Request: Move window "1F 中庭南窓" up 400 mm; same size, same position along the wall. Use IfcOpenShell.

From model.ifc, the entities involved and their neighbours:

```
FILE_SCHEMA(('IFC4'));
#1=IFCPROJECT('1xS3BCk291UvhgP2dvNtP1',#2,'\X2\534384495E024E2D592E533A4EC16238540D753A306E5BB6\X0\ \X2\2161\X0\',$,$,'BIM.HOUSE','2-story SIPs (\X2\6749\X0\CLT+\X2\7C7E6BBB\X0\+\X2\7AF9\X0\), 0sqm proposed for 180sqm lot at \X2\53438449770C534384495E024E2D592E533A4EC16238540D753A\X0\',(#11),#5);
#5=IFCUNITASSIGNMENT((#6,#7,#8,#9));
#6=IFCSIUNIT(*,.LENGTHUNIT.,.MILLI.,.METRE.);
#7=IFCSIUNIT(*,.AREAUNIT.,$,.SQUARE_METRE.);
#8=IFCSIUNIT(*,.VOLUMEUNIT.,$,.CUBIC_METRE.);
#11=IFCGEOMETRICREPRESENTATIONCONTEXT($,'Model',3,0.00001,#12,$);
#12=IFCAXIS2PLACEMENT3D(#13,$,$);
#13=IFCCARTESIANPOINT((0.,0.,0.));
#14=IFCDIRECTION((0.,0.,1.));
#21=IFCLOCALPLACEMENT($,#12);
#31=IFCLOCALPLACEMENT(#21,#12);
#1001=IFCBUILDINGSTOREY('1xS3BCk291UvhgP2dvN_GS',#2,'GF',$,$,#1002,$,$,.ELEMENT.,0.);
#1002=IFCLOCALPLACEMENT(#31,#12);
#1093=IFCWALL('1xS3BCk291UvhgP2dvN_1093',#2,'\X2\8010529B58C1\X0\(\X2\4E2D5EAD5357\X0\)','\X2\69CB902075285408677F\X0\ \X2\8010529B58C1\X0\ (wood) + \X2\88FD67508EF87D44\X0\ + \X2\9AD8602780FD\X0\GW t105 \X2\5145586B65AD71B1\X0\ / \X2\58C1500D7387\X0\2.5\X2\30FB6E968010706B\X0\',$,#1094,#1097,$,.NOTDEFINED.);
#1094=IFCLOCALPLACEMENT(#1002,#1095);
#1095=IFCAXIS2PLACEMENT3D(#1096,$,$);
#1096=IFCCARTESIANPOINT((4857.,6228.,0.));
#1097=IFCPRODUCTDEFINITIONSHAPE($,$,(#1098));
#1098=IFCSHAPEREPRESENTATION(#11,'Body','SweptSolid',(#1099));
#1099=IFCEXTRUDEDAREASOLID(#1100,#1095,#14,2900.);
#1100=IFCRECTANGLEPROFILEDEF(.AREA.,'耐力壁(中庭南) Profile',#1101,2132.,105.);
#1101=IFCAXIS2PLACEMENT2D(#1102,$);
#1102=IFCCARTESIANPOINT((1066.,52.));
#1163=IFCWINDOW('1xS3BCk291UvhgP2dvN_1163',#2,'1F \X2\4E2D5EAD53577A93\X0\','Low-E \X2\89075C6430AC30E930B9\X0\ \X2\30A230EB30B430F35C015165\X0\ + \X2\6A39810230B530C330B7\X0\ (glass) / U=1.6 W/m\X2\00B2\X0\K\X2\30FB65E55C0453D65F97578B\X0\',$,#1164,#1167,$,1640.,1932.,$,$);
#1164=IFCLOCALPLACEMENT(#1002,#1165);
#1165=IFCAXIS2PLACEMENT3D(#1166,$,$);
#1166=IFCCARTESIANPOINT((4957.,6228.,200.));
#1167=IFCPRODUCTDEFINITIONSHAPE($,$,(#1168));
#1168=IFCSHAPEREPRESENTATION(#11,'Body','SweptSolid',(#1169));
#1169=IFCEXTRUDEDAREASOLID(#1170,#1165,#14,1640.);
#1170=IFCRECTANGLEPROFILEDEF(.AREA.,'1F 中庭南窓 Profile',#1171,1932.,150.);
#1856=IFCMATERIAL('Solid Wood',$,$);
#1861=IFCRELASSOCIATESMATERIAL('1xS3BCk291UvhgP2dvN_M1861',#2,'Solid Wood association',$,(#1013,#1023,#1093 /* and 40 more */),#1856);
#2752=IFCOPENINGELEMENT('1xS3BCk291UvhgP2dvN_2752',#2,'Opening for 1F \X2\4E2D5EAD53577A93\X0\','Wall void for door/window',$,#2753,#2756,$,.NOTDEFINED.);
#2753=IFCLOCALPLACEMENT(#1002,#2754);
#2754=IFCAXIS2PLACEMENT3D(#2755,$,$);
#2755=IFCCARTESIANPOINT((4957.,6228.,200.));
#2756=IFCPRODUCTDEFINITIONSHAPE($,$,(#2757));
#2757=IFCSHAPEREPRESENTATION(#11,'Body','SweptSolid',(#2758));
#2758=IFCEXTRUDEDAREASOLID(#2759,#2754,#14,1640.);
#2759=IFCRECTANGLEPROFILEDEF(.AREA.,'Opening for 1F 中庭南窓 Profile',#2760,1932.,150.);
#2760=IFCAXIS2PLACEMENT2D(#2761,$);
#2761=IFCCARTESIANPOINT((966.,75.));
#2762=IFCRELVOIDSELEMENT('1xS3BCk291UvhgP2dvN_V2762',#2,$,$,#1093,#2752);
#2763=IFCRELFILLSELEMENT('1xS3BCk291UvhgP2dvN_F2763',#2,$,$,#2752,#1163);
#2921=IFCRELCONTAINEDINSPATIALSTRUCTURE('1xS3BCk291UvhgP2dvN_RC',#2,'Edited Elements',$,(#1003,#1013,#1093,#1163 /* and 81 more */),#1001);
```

```python
import numpy as np
import ifcopenshell
import ifcopenshell.api.geometry
import ifcopenshell.util.placement
import ifcopenshell.util.unit

model = ifcopenshell.open("model.ifc")
unit_scale = ifcopenshell.util.unit.calculate_unit_scale(model)

window = model.by_id(1163)
opening = window.FillsVoids[0].RelatingOpeningElement
dz = 400.0

shift = np.array([0.0, 0.0, dz])
# The window is not placed relative to its opening, so move both.
for product in (opening, window):
    matrix = ifcopenshell.util.placement.get_local_placement(product.ObjectPlacement)
    matrix[:3, 3] += shift
    ifcopenshell.api.geometry.edit_object_placement(model, product=product, matrix=matrix, is_si=False)

print(f"moved by {dz * unit_scale:+.3f} m")

model.write("model_edited.ifc")
```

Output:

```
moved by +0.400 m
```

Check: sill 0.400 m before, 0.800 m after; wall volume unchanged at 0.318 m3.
